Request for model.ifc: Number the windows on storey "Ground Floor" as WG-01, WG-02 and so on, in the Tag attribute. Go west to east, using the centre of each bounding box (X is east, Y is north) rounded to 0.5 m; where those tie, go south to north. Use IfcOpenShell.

First a look at what the model holds.

```python
import ifcopenshell
import ifcopenshell.util.element
import ifcopenshell.util.placement

model = ifcopenshell.open("model.ifc")
print(model.schema)
storey = next(s for s in model.by_type("IfcBuildingStorey") if s.Name == "Ground Floor")
windows = [e for e in ifcopenshell.util.element.get_decomposition(storey) if e.is_a("IfcWindow")]
for e in sorted(windows, key=lambda e: e.id()):
    origin = ifcopenshell.util.placement.get_local_placement(e.ObjectPlacement)[:3, 3]
    print(e.id(), e.Tag, e.Name, origin.round(2) + 0.0, sep=" | ")
```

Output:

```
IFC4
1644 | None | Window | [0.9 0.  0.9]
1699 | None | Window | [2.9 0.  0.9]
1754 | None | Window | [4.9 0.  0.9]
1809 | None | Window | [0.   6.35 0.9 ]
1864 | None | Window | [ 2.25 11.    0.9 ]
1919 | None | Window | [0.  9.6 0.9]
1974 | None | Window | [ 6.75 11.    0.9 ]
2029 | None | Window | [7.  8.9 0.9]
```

```python
import ifcopenshell
import ifcopenshell.geom
import ifcopenshell.util.element
import ifcopenshell.util.shape

model = ifcopenshell.open("model.ifc")
settings = ifcopenshell.geom.settings()
settings.set("use-world-coords", True)


def centre(element):
    shape = ifcopenshell.geom.create_shape(settings, element)
    return ifcopenshell.util.shape.get_bbox_centroid(shape.geometry)


storey = next(s for s in model.by_type("IfcBuildingStorey") if s.Name == "Ground Floor")
windows = [e for e in ifcopenshell.util.element.get_decomposition(storey) if e.is_a("IfcWindow")]

# Insertion points can sit at a corner or the storey origin, so sort by the geometry (in metres).
centres = {e: centre(e) for e in windows}
windows.sort(key=lambda e: (round(centres[e][0] / 0.5), centres[e][1]))

for i, e in enumerate(windows, start=1):
    number = f"WG-{i:02d}"
    e.Tag = number
    print(e.id(), number)

model.write("model_v2.ifc")
```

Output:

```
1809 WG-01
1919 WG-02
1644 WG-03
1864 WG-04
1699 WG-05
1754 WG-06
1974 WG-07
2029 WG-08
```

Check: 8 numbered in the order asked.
